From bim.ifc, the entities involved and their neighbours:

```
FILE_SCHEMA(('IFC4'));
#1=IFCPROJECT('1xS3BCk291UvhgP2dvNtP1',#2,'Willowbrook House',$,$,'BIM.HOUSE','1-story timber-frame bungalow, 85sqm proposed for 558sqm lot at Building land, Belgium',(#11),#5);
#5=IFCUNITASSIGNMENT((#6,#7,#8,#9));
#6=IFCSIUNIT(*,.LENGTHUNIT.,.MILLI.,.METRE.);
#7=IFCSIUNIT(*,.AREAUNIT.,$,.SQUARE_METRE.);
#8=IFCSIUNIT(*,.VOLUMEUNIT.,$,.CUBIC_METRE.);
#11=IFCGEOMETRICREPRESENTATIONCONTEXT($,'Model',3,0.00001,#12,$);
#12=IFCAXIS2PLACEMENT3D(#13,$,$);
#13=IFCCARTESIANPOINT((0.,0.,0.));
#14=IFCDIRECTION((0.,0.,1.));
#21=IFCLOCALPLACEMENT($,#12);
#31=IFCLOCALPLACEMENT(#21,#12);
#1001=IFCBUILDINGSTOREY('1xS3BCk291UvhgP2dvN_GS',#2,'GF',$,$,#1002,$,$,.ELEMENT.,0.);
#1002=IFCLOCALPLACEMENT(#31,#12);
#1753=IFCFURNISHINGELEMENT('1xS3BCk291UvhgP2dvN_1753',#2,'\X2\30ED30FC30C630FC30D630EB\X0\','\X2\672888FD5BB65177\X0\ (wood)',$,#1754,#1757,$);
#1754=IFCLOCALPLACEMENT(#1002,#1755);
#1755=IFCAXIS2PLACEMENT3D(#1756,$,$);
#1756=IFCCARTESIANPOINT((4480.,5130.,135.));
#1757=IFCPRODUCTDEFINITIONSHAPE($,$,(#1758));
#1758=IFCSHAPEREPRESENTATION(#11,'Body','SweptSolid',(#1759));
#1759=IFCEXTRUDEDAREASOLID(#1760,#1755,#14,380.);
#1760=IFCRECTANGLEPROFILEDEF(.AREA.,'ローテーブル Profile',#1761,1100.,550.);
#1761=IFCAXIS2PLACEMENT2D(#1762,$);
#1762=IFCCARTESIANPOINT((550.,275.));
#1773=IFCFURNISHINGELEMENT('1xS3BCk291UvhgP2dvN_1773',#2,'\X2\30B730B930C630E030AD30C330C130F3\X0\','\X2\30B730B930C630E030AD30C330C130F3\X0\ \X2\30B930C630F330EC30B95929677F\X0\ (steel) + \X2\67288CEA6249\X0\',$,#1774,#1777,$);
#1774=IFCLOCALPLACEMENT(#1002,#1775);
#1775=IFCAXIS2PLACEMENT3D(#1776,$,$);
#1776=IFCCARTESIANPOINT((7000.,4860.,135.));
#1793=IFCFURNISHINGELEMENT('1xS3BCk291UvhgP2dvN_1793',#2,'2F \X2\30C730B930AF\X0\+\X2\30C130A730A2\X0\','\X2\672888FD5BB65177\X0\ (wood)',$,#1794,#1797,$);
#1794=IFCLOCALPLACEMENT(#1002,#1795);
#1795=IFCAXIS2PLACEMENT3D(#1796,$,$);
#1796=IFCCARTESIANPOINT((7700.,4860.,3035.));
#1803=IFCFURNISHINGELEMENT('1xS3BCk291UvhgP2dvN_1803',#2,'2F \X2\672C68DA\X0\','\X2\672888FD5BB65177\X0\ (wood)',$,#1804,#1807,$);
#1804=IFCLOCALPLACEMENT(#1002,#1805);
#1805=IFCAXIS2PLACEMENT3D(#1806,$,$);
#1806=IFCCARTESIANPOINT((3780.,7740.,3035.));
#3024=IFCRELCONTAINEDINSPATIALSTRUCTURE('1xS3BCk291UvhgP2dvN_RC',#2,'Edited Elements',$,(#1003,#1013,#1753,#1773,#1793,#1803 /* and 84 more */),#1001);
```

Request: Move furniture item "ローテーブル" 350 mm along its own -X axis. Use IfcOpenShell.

```python
import ifcopenshell
import ifcopenshell.api.geometry
import ifcopenshell.util.placement

model = ifcopenshell.open("bim.ifc")

item = model.by_id(1753)
matrix = ifcopenshell.util.placement.get_local_placement(item.ObjectPlacement)
matrix[:3, 3] -= matrix[:3, 0] * 350.0
ifcopenshell.api.geometry.edit_object_placement(model, product=item, matrix=matrix, is_si=False)

print(ifcopenshell.util.placement.get_local_placement(item.ObjectPlacement).round(3) + 0.0)

model.write("bim_rev.ifc")
```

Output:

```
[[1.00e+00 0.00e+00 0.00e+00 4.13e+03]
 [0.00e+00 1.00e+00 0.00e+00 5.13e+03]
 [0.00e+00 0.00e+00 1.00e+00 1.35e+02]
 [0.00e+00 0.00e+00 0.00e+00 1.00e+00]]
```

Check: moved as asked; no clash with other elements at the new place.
